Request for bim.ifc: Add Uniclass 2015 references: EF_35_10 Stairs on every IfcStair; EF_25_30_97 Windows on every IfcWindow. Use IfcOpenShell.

First a look at what the model holds.

```python
import ifcopenshell

model = ifcopenshell.open("bim.ifc")
print(model.schema)
print("classifications:", [c.Name for c in model.by_type("IfcClassification")])
for ifc_class in ("IfcDoor", "IfcRoof", "IfcStair", "IfcWall", "IfcWindow"):
    print(ifc_class, len(model.by_type(ifc_class)))
```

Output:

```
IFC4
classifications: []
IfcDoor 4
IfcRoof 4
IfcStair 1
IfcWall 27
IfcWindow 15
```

```python
import ifcopenshell
import ifcopenshell.api.classification

model = ifcopenshell.open("bim.ifc")

system = ifcopenshell.api.classification.add_classification(model, classification="Uniclass 2015")

codes = {
    "IfcStair": ("EF_35_10", "Stairs"),
    "IfcWindow": ("EF_25_30_97", "Windows"),
}
for ifc_class, (code, name) in codes.items():
    products = model.by_type(ifc_class)
    ifcopenshell.api.classification.add_reference(
        model, products=products, classification=system, identification=code, name=name
    )
    print(code, len(products))

model.write("bim_updated.ifc")
```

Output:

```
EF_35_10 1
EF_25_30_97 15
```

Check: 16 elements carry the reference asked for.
